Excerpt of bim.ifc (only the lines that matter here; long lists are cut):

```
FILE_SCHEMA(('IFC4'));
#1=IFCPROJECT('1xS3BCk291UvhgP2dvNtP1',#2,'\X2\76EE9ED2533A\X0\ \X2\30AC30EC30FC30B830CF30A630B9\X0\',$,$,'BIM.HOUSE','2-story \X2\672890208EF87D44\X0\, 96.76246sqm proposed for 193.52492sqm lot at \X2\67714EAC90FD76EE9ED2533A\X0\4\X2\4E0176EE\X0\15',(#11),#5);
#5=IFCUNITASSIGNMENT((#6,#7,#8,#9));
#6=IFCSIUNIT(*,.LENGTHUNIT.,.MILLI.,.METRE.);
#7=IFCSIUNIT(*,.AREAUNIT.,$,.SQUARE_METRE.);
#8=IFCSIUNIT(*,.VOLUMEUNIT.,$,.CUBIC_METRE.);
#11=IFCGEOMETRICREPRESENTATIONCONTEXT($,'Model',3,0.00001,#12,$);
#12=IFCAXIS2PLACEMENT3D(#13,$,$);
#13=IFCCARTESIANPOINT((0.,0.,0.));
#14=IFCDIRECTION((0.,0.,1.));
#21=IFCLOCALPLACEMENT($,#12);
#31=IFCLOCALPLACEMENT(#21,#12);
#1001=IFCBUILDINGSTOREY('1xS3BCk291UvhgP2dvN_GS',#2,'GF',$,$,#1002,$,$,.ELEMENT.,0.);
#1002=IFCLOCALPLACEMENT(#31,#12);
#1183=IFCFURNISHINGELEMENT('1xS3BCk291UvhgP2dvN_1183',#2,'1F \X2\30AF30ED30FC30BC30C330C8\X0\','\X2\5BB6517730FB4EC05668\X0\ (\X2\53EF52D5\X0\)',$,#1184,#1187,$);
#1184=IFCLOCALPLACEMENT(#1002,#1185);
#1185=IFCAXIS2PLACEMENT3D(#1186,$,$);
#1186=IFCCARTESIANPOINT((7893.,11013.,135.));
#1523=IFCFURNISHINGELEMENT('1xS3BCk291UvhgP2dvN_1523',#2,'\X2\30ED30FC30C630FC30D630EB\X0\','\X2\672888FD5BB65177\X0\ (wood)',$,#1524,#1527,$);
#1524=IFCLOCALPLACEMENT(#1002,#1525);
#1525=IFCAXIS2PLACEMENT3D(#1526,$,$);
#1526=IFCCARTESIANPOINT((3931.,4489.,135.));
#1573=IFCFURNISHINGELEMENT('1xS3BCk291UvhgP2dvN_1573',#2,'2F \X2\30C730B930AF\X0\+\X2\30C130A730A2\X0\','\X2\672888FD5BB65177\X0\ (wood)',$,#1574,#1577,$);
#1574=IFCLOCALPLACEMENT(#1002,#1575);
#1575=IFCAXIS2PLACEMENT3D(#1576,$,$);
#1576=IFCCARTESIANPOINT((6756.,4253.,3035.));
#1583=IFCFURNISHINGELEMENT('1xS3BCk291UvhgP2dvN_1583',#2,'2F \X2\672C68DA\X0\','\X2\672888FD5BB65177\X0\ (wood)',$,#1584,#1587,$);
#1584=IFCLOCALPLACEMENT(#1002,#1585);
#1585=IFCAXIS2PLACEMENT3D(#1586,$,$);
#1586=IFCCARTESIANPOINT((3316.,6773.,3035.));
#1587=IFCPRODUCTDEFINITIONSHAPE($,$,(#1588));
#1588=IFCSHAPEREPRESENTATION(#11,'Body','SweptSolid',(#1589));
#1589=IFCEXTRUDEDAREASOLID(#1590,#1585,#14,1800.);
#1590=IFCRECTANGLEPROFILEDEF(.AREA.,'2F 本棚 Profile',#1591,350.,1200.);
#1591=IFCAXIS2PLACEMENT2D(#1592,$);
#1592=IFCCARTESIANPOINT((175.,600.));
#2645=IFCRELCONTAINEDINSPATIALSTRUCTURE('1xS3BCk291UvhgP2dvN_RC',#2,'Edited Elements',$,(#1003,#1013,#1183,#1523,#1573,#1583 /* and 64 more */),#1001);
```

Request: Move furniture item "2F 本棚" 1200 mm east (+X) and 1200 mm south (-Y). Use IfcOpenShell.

```python
import ifcopenshell
import ifcopenshell.api.geometry
import ifcopenshell.util.placement
import ifcopenshell.util.unit

model = ifcopenshell.open("bim.ifc")
unit_scale = ifcopenshell.util.unit.calculate_unit_scale(model)

item = model.by_id(1583)
matrix = ifcopenshell.util.placement.get_local_placement(item.ObjectPlacement)
matrix[0, 3] += 1.2 / unit_scale
matrix[1, 3] -= 1.2 / unit_scale
ifcopenshell.api.geometry.edit_object_placement(model, product=item, matrix=matrix, is_si=False)

print(ifcopenshell.util.placement.get_local_placement(item.ObjectPlacement).round(3) + 0.0)

model.write("bim_rev.ifc")
```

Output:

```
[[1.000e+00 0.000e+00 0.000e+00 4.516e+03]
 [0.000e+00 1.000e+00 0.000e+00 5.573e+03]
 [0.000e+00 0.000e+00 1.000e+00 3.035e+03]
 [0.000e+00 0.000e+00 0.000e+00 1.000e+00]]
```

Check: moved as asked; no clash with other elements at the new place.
